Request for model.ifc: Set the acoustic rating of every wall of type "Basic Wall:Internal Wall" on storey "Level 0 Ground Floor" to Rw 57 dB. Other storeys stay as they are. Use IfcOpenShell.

First a look at what the model holds.

```python
import ifcopenshell
import ifcopenshell.util.element

model = ifcopenshell.open("model.ifc")
print(model.schema)
storey = next(s for s in model.by_type("IfcBuildingStorey") if s.Name == "Level 0 Ground Floor")
walls = [e for e in ifcopenshell.util.element.get_decomposition(storey) if e.is_a("IfcWall")]
seen = {}
for e in walls:
    element_type = ifcopenshell.util.element.get_type(e)
    key = (element_type.Name if element_type != e and element_type else None, ifcopenshell.util.element.get_pset(e, "Pset_WallCommon", "AcousticRating"))
    seen[key] = seen.get(key, 0) + 1
for (name, value), count in sorted(seen.items(), key=str):
    print(count, "x", name, "|", value)
```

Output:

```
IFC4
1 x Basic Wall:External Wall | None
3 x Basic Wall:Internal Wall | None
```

```python
import ifcopenshell
import ifcopenshell.api.pset
import ifcopenshell.util.element

model = ifcopenshell.open("model.ifc")

storey = next(s for s in model.by_type("IfcBuildingStorey") if s.Name == "Level 0 Ground Floor")
walls = [e for e in ifcopenshell.util.element.get_decomposition(storey) if e.is_a("IfcWall")]

count = 0
for e in walls:
    element_type = ifcopenshell.util.element.get_type(e)
    if element_type in (None, e) or element_type.Name != "Basic Wall:Internal Wall":
        continue
    # add_pset returns the element's existing set when there is one.
    pset = ifcopenshell.api.pset.add_pset(model, product=e, name="Pset_WallCommon")
    ifcopenshell.api.pset.edit_pset(model, pset=pset, properties={"AcousticRating": "Rw 57 dB"})
    count += 1

print(count, "walls updated")

model.write("model_rev.ifc")
```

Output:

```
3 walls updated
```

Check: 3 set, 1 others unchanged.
